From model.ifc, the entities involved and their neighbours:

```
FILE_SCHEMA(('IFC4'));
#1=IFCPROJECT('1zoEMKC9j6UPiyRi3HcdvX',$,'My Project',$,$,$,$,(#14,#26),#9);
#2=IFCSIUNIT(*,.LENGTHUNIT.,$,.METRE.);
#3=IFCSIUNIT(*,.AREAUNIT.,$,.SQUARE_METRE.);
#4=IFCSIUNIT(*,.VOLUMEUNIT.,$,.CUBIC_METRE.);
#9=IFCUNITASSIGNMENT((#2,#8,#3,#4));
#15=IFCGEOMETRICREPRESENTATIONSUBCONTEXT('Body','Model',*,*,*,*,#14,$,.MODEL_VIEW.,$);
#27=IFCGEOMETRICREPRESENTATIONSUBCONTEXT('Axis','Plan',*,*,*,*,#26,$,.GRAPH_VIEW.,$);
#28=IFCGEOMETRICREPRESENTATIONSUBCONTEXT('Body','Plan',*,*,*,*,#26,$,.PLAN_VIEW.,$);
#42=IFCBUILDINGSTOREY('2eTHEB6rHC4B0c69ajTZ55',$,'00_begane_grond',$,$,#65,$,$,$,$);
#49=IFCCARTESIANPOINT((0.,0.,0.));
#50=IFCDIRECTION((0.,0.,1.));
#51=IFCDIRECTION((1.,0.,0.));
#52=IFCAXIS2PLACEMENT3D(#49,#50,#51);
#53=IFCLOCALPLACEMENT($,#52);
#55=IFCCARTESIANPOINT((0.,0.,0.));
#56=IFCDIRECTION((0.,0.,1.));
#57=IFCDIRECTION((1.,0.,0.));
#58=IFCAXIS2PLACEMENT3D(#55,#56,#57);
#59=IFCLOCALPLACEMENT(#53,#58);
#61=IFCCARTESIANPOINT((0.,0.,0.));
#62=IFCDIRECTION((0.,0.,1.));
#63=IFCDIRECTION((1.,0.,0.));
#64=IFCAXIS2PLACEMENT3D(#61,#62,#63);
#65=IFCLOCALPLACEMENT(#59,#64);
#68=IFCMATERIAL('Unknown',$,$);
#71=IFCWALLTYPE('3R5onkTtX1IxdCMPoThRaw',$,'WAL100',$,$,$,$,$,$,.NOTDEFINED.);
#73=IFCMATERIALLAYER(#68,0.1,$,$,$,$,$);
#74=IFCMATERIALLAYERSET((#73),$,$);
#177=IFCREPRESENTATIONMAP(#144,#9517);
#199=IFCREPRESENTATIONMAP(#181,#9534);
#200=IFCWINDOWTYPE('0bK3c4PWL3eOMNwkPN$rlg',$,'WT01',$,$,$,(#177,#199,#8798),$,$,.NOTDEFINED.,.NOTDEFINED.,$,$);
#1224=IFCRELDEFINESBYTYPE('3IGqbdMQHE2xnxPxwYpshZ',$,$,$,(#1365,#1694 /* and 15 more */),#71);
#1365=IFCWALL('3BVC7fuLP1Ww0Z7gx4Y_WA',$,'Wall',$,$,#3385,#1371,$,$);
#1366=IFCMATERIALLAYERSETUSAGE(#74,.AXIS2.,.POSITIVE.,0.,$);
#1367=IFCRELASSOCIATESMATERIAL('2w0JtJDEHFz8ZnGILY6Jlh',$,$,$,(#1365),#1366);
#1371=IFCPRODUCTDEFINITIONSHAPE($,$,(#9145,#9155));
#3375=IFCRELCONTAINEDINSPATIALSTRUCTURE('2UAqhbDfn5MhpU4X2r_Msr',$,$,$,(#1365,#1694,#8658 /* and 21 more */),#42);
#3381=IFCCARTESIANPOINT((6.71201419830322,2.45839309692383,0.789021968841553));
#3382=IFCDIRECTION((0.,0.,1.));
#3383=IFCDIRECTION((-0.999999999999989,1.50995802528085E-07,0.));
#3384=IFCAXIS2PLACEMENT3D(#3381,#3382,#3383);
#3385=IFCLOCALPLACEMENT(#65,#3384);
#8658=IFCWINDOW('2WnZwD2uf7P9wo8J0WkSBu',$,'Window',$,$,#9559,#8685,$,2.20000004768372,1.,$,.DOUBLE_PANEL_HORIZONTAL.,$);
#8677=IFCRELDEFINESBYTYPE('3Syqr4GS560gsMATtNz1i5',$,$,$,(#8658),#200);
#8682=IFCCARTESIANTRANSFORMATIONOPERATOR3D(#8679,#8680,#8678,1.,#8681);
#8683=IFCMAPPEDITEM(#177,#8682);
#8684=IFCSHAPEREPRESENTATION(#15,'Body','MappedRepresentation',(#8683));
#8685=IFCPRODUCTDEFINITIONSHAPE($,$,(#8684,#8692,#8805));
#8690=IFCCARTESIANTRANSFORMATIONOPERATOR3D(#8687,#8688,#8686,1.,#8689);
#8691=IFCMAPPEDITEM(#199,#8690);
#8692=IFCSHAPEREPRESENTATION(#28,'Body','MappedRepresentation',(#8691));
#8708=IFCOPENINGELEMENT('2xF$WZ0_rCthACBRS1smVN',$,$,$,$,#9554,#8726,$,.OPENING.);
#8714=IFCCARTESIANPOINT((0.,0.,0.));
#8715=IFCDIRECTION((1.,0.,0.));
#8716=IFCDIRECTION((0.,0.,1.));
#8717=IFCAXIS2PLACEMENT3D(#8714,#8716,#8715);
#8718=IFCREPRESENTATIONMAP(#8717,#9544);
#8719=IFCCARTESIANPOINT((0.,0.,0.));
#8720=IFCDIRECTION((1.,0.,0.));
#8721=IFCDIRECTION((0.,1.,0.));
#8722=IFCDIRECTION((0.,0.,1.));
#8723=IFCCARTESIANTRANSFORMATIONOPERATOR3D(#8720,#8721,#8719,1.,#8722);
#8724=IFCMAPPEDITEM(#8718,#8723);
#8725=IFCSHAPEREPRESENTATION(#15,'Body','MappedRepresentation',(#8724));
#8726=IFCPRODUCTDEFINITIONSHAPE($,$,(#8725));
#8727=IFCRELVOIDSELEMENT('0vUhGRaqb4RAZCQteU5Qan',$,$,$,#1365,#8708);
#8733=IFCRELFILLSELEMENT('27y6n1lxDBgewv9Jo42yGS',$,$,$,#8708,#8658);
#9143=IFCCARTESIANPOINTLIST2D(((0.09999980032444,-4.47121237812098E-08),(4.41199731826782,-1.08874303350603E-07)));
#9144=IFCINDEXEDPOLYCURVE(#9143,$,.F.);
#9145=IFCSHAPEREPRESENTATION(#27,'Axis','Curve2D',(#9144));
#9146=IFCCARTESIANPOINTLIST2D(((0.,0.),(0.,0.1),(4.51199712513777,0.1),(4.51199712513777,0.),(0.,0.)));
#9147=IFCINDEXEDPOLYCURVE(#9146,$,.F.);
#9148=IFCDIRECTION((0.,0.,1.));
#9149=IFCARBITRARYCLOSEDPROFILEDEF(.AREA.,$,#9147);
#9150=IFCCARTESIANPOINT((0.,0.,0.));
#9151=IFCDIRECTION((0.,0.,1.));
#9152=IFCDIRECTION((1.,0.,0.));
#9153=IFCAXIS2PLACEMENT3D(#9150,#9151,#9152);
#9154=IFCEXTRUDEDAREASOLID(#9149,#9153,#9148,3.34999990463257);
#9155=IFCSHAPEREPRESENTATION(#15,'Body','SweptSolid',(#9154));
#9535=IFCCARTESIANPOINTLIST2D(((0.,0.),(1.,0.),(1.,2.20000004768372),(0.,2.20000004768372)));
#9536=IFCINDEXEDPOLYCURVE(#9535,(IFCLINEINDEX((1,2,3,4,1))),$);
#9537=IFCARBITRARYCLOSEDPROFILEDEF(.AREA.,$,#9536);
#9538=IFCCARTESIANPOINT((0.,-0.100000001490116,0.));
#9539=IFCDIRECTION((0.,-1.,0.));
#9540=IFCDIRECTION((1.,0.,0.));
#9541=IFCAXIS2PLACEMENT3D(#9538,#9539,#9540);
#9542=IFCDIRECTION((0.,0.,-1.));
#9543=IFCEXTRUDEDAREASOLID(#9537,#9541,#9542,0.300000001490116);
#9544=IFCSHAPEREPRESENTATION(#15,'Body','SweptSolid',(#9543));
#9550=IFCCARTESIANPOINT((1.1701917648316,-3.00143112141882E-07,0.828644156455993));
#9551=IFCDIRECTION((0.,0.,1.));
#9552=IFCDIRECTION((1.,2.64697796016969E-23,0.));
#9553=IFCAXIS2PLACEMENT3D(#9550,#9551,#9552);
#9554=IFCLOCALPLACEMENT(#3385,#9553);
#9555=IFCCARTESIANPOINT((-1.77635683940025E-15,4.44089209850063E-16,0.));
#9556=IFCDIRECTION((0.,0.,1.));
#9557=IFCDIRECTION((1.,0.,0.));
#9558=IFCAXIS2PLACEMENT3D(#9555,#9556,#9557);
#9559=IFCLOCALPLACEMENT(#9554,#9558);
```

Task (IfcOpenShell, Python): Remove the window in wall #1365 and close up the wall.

```python
import ifcopenshell
import ifcopenshell.api.feature
import ifcopenshell.api.root
import ifcopenshell.geom
import ifcopenshell.util.shape

model = ifcopenshell.open("model.ifc")
settings = ifcopenshell.geom.settings()


def volume(element):
    """Net volume in cubic metres, openings subtracted."""
    shape = ifcopenshell.geom.create_shape(settings, element)
    return ifcopenshell.util.shape.get_volume(shape.geometry)


window = model.by_guid("2WnZwD2uf7P9wo8J0WkSBu")
opening = window.FillsVoids[0].RelatingOpeningElement
wall = opening.VoidsElements[0].RelatingBuildingElement
before = volume(wall)

ifcopenshell.api.root.remove_product(model, product=window)
ifcopenshell.api.feature.remove_feature(model, feature=opening)

after = volume(wall)

print(f"wall volume {before:.3f} -> {after:.3f} m3")

model.write("model_rev.ifc")
```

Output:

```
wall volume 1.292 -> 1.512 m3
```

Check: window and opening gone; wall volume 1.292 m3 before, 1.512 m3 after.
